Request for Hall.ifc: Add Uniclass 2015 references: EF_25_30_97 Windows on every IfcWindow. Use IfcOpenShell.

First a look at what the model holds.

```python
import ifcopenshell

model = ifcopenshell.open("Hall.ifc")
print(model.schema)
print("classifications:", [c.Name for c in model.by_type("IfcClassification")])
for ifc_class in ("IfcDoor", "IfcRoof", "IfcStair", "IfcWall", "IfcWindow"):
    print(ifc_class, len(model.by_type(ifc_class)))
```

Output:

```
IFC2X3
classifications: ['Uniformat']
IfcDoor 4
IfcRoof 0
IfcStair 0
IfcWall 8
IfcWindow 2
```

```python
import ifcopenshell
import ifcopenshell.api.classification

model = ifcopenshell.open("Hall.ifc")

# IFC2X3 requires Source and Edition and has no link from the project to the system.
system = model.create_entity("IfcClassification", Source="NBS", Edition="2015", Name="Uniclass 2015")

codes = {
    "IfcWindow": ("EF_25_30_97", "Windows"),
}
for ifc_class, (code, name) in codes.items():
    products = model.by_type(ifc_class)
    ifcopenshell.api.classification.add_reference(
        model, products=products, classification=system, identification=code, name=name
    )
    print(code, len(products))

model.write("Hall_updated.ifc")
```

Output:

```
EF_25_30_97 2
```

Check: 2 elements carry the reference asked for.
